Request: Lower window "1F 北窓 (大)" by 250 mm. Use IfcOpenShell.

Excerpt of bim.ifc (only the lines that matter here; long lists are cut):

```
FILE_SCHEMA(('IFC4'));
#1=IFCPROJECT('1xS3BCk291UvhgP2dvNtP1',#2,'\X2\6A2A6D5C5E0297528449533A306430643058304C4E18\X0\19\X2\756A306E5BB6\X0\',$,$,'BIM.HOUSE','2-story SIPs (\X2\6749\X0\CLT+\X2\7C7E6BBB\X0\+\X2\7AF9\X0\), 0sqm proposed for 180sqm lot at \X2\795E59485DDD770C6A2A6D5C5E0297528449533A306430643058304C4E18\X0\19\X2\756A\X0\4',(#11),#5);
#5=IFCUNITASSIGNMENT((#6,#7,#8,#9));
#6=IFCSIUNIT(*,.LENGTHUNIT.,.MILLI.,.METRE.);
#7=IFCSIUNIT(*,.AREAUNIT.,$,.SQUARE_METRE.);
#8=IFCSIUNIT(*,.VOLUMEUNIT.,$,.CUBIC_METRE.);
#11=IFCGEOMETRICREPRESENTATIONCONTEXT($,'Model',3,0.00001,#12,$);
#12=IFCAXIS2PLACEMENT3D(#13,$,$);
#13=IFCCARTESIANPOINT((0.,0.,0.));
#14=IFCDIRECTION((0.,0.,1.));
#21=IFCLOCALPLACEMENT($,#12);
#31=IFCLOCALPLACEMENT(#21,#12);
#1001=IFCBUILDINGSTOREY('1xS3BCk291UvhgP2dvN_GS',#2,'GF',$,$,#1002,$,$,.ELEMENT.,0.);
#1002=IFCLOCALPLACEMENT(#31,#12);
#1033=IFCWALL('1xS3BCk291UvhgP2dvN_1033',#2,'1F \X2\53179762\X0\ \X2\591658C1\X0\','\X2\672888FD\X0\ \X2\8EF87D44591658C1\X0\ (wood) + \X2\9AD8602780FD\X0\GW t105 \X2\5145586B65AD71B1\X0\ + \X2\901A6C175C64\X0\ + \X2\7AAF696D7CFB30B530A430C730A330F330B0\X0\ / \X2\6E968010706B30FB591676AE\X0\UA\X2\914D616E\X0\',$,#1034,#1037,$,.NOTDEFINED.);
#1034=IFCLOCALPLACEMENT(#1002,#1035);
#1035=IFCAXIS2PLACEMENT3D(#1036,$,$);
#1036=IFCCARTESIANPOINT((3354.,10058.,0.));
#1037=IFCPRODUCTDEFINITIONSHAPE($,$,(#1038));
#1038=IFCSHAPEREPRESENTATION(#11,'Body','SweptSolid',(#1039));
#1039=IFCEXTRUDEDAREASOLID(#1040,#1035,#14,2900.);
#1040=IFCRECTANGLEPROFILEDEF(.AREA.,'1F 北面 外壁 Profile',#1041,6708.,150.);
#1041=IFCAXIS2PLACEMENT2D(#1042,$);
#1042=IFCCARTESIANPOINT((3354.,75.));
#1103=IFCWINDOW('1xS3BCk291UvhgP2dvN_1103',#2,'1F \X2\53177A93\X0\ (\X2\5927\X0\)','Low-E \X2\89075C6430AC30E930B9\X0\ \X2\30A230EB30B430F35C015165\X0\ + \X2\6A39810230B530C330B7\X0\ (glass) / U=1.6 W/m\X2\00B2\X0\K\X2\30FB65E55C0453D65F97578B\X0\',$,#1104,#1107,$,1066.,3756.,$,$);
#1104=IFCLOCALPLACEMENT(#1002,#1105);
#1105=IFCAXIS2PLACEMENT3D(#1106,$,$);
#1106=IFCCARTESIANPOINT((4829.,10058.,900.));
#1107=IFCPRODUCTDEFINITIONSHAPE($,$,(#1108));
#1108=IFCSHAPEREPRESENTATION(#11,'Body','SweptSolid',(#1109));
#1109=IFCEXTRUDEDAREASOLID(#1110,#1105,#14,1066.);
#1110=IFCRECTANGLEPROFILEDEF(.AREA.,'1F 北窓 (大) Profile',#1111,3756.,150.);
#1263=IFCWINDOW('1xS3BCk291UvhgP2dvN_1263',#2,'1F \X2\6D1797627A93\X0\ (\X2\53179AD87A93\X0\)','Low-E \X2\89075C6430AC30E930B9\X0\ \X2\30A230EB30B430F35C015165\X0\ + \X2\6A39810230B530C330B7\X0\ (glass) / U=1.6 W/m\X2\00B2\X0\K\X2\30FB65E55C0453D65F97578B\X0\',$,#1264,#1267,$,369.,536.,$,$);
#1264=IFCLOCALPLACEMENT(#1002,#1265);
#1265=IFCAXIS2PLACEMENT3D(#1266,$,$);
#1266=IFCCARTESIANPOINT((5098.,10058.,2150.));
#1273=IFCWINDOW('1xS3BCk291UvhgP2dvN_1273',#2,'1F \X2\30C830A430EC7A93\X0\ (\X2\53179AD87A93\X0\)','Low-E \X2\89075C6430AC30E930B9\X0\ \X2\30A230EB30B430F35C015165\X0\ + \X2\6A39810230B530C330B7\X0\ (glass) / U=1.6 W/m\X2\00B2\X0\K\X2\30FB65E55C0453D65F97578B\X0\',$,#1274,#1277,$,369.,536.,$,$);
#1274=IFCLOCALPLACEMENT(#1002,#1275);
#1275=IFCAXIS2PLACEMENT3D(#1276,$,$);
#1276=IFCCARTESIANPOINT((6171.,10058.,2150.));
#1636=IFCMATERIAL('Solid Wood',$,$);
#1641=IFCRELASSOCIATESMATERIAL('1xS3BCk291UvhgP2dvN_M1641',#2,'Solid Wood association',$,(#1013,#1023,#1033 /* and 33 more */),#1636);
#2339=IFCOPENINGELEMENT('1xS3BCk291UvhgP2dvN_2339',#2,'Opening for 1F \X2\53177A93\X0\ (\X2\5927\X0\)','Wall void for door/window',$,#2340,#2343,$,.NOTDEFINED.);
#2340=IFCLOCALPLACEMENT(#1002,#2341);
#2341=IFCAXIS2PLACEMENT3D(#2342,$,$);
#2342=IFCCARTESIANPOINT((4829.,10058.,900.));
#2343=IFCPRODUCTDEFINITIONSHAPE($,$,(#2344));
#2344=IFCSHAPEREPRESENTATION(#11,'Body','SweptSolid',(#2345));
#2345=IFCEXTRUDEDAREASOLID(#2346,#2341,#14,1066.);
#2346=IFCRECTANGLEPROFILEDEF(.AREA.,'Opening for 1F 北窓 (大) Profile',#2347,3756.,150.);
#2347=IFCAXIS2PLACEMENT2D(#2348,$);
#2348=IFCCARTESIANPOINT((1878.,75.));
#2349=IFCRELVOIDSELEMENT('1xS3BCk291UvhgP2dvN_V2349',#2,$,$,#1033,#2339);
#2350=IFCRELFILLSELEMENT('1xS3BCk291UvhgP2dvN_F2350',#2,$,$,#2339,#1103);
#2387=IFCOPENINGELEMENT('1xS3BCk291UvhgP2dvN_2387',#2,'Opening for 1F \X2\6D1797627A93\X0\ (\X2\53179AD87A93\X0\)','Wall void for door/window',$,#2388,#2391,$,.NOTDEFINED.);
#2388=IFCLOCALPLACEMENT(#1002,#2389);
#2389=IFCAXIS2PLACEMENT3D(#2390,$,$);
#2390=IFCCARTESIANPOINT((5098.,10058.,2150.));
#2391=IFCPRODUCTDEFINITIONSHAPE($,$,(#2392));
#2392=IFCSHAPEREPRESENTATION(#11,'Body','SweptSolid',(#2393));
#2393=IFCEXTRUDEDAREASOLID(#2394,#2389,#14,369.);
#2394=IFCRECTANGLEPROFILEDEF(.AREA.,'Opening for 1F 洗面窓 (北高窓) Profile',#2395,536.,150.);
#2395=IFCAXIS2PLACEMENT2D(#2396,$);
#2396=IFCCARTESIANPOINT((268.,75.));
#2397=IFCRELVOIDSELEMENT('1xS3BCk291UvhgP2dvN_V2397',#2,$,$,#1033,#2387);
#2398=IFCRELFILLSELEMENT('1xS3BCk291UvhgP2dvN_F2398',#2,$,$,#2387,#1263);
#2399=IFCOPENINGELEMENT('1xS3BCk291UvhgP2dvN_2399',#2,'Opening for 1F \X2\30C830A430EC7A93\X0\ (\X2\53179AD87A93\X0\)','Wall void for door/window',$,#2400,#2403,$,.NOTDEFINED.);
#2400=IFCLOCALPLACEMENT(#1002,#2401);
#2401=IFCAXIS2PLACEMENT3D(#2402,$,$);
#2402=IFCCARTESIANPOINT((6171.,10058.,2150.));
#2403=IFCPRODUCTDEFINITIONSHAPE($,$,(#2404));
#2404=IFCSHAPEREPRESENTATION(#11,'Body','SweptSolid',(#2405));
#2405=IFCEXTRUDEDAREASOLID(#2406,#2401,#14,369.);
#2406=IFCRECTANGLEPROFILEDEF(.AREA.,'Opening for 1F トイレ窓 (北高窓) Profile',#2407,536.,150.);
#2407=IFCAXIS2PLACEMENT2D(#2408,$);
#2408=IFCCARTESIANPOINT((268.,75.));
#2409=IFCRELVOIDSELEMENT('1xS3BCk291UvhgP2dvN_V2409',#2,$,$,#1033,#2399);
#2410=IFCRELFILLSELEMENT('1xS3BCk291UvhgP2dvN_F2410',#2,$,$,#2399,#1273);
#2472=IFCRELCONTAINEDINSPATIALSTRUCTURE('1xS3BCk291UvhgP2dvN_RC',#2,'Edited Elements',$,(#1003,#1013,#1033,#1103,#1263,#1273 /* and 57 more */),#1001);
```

```python
import numpy as np
import ifcopenshell
import ifcopenshell.api.geometry
import ifcopenshell.util.placement
import ifcopenshell.util.unit

model = ifcopenshell.open("bim.ifc")
unit_scale = ifcopenshell.util.unit.calculate_unit_scale(model)

window = model.by_id(1103)
opening = window.FillsVoids[0].RelatingOpeningElement
dz = -0.25 / unit_scale

shift = np.array([0.0, 0.0, dz])
# The window is not placed relative to its opening, so move both.
for product in (opening, window):
    matrix = ifcopenshell.util.placement.get_local_placement(product.ObjectPlacement)
    matrix[:3, 3] += shift
    ifcopenshell.api.geometry.edit_object_placement(model, product=product, matrix=matrix, is_si=False)

print(f"moved by {dz * unit_scale:+.3f} m")

model.write("bim_updated.ifc")
```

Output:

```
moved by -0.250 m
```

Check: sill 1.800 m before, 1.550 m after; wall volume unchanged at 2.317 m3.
